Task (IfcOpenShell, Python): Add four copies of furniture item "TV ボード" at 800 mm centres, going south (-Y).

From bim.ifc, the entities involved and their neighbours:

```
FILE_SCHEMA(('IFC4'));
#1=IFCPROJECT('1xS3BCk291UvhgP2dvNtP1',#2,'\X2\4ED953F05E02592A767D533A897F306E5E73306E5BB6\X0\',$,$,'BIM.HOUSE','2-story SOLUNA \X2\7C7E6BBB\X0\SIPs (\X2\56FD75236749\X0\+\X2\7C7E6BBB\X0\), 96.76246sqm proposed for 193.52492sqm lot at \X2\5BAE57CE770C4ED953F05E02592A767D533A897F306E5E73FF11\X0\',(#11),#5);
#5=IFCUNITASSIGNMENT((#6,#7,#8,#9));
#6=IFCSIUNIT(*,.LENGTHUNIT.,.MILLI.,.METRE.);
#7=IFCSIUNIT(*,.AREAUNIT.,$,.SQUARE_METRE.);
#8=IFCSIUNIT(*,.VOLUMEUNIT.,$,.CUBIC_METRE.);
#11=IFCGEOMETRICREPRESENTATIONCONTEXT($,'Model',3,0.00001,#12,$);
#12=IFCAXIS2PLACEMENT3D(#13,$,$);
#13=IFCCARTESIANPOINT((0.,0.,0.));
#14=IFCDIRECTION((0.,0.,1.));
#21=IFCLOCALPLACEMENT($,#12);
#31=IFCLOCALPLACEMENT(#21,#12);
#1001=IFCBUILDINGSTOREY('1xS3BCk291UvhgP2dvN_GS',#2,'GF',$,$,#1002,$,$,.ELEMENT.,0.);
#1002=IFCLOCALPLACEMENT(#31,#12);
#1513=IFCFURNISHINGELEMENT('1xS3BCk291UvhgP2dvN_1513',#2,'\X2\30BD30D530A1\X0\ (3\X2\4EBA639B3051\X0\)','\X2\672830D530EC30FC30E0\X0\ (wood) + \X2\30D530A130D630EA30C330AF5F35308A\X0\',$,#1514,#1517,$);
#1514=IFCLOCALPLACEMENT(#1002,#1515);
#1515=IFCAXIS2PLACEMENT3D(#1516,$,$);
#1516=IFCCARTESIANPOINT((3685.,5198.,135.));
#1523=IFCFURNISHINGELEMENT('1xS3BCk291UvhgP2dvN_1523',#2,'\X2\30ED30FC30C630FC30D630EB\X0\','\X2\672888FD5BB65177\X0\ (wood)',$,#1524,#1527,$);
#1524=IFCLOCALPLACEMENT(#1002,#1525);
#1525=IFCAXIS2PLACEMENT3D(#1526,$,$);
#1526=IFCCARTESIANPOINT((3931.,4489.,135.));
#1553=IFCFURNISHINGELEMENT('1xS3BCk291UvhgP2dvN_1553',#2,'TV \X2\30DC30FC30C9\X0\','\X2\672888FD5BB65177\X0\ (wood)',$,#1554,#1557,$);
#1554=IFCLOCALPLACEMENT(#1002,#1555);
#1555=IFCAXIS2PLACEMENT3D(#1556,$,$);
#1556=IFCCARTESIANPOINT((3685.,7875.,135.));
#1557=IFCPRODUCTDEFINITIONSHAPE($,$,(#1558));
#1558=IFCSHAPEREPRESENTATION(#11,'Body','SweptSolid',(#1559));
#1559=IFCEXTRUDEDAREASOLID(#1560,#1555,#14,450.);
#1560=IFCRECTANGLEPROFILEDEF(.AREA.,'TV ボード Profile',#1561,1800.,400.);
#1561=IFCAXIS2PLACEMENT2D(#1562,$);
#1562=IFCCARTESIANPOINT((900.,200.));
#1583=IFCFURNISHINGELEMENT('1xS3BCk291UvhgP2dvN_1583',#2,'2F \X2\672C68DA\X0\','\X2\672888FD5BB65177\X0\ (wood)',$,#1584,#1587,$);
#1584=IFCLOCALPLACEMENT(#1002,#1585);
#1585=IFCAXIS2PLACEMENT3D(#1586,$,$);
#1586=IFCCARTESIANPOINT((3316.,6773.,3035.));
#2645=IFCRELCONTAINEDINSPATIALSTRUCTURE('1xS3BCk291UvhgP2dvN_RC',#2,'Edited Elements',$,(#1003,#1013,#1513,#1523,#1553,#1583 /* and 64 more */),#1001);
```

```python
import numpy as np
import ifcopenshell
import ifcopenshell.api.geometry
import ifcopenshell.api.root
import ifcopenshell.util.element
import ifcopenshell.util.placement

model = ifcopenshell.open("bim.ifc")


def reuse_history(source, copy):
    """copy_class also copies each property set's owner history, people and application; keep the originals."""
    for rel in copy.IsDefinedBy:
        if rel.is_a("IfcRelDefinesByProperties") and (history := rel.RelatingPropertyDefinition.OwnerHistory):
            rel.RelatingPropertyDefinition.OwnerHistory = source.OwnerHistory
            ifcopenshell.util.element.remove_deep2(model, history)


source = model.by_id(1553)
base = ifcopenshell.util.placement.get_local_placement(source.ObjectPlacement)
step = np.array([0.0, -1.0, 0.0]) * 800.0

for i in range(1, 5):
    copy = ifcopenshell.api.root.copy_class(model, product=source)
    copy.Representation = ifcopenshell.util.element.copy_deep(
        model, source.Representation, exclude=["IfcGeometricRepresentationContext", "IfcRepresentationMap"]
    )
    reuse_history(source, copy)
    matrix = base.copy()
    matrix[:3, 3] += i * step
    print("added at", matrix[:3, 3].round(3) + 0.0)
    ifcopenshell.api.geometry.edit_object_placement(model, product=copy, matrix=matrix, is_si=False)

model.write("bim_v2.ifc")
```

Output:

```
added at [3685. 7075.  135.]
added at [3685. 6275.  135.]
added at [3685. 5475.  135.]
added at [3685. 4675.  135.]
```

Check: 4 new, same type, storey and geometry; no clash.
